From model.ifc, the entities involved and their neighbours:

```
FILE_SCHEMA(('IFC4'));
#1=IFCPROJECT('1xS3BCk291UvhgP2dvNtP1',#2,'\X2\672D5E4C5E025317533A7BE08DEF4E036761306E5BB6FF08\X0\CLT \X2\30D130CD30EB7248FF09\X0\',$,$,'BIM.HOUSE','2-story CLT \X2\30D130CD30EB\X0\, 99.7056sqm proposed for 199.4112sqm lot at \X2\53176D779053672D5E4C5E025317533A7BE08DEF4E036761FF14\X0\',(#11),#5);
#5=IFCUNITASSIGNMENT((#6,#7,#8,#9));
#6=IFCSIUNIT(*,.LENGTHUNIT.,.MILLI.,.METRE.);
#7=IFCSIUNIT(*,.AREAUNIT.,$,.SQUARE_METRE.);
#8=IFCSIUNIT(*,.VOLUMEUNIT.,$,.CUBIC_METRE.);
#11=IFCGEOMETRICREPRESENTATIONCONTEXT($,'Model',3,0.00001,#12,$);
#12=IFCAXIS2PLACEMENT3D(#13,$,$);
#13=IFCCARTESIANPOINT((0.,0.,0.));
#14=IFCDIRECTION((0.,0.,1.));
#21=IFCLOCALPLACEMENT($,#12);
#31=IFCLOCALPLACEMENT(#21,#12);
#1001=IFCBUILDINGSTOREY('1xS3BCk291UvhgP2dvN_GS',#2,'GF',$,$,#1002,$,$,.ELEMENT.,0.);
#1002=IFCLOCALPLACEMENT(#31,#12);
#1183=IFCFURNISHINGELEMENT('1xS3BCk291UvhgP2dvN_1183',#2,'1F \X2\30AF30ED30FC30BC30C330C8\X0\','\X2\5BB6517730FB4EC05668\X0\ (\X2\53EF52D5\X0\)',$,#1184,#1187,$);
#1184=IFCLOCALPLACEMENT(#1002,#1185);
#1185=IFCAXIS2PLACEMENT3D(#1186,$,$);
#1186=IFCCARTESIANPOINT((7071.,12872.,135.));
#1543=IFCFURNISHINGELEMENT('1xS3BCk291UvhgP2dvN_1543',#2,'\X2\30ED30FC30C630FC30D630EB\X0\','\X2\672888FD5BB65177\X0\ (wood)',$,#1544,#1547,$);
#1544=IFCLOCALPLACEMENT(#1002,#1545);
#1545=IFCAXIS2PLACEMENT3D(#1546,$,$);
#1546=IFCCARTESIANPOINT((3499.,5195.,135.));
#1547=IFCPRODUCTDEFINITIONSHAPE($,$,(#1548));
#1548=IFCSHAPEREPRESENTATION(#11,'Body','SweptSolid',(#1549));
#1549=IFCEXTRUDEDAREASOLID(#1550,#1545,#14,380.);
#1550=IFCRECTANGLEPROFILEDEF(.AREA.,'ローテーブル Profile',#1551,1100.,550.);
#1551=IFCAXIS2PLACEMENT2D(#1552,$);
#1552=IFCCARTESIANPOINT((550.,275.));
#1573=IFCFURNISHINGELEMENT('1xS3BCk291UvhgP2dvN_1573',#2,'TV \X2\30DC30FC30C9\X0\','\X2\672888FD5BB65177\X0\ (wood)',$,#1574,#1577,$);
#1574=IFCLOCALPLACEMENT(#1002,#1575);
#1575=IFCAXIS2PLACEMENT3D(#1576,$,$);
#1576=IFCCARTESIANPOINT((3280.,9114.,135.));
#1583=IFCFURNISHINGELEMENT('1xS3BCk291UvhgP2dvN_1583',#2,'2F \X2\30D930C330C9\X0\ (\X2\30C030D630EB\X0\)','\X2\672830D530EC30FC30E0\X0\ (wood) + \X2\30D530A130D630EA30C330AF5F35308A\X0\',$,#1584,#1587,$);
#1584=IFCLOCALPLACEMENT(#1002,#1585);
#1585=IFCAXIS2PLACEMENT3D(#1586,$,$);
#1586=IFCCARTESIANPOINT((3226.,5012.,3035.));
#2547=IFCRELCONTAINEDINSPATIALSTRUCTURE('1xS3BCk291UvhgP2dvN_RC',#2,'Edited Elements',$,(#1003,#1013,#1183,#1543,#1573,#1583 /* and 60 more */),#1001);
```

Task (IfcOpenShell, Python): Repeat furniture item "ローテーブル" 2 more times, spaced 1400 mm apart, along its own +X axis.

```python
import ifcopenshell
import ifcopenshell.api.geometry
import ifcopenshell.api.root
import ifcopenshell.util.element
import ifcopenshell.util.placement
import ifcopenshell.util.unit

model = ifcopenshell.open("model.ifc")
unit_scale = ifcopenshell.util.unit.calculate_unit_scale(model)


def reuse_history(source, copy):
    """copy_class also copies each property set's owner history, people and application; keep the originals."""
    for rel in copy.IsDefinedBy:
        if rel.is_a("IfcRelDefinesByProperties") and (history := rel.RelatingPropertyDefinition.OwnerHistory):
            rel.RelatingPropertyDefinition.OwnerHistory = source.OwnerHistory
            ifcopenshell.util.element.remove_deep2(model, history)


source = model.by_guid("1xS3BCk291UvhgP2dvN_1543")
base = ifcopenshell.util.placement.get_local_placement(source.ObjectPlacement)
step = base[:3, 0] * 1.4 / unit_scale

for i in range(1, 3):
    copy = ifcopenshell.api.root.copy_class(model, product=source)
    copy.Representation = ifcopenshell.util.element.copy_deep(
        model, source.Representation, exclude=["IfcGeometricRepresentationContext", "IfcRepresentationMap"]
    )
    reuse_history(source, copy)
    matrix = base.copy()
    matrix[:3, 3] += i * step
    print("added at", matrix[:3, 3].round(3) + 0.0)
    ifcopenshell.api.geometry.edit_object_placement(model, product=copy, matrix=matrix, is_si=False)

model.write("model_updated.ifc")
```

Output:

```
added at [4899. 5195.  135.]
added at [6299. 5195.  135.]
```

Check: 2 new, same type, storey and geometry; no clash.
